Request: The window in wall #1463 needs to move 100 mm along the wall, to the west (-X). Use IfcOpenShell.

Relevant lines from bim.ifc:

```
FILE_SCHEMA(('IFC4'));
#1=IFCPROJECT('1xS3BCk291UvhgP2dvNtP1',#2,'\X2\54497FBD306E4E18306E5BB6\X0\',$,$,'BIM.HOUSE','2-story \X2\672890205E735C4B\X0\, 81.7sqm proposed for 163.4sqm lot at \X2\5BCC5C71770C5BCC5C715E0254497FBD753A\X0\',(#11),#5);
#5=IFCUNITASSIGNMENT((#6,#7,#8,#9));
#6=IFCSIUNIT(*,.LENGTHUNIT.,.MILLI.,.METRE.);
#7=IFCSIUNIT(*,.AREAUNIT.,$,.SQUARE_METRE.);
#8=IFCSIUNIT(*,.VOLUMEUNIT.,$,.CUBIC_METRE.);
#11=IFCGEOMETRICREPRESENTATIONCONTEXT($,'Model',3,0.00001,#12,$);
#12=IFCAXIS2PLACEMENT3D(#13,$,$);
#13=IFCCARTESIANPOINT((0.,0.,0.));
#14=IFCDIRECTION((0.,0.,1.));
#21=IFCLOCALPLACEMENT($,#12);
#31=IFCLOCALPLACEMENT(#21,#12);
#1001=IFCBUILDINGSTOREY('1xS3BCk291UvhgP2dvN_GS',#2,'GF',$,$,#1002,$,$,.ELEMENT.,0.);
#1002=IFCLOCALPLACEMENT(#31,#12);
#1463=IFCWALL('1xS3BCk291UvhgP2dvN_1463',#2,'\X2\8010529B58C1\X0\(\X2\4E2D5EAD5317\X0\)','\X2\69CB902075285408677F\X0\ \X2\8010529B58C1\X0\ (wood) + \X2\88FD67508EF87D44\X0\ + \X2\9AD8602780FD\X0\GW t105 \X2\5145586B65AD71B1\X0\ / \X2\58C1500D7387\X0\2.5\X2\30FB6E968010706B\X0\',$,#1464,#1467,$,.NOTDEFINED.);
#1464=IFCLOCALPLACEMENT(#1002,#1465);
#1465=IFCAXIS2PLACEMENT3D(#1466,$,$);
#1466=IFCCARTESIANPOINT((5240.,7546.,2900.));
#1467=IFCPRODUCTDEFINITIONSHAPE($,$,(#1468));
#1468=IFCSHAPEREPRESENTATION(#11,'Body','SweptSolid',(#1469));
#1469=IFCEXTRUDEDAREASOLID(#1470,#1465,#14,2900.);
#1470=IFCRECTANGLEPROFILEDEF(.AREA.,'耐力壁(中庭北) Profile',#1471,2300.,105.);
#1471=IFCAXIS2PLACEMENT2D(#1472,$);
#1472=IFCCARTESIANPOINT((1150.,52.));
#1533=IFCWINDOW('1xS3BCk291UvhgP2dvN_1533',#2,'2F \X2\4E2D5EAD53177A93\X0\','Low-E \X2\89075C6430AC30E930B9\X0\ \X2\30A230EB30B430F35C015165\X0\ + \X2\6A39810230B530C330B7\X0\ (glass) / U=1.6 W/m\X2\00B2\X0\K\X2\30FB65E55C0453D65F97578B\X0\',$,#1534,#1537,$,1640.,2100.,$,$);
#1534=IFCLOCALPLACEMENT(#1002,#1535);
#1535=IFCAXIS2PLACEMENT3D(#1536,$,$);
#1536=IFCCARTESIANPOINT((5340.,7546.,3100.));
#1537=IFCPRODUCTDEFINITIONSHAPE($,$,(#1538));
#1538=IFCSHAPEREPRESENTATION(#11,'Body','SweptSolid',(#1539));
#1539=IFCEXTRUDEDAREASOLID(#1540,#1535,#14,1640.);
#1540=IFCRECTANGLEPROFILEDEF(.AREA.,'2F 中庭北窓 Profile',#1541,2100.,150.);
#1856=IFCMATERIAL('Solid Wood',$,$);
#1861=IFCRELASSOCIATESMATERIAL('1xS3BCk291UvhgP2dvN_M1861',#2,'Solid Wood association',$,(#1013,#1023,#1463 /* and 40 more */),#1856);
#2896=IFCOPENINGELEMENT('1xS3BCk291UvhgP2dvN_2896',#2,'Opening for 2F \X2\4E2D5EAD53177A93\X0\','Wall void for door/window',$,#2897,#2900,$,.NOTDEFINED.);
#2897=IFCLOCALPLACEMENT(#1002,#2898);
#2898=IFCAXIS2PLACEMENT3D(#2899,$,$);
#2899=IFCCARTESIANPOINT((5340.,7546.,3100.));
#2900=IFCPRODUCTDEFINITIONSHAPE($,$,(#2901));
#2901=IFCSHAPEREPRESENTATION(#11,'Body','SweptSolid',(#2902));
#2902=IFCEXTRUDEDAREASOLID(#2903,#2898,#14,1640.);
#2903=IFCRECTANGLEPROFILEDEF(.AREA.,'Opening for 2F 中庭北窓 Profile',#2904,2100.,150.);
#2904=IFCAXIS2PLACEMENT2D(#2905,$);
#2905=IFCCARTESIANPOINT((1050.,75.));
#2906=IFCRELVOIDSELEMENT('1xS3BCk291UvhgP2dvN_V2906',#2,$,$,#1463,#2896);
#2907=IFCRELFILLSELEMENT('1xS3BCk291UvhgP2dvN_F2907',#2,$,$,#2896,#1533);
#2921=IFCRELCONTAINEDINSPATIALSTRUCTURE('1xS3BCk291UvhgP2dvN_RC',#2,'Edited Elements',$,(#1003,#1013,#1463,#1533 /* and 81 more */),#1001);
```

```python
import ifcopenshell
import ifcopenshell.api.geometry
import ifcopenshell.util.placement
import ifcopenshell.util.unit

model = ifcopenshell.open("bim.ifc")
unit_scale = ifcopenshell.util.unit.calculate_unit_scale(model)

window = model.by_id(1533)
opening = window.FillsVoids[0].RelatingOpeningElement
wall = opening.VoidsElements[0].RelatingBuildingElement

wall_matrix = ifcopenshell.util.placement.get_local_placement(wall.ObjectPlacement)
shift = wall_matrix[:3, 0] * -0.1 / unit_scale
before = ifcopenshell.util.placement.get_local_placement(window.ObjectPlacement)[:3, 3].copy()

# The window is not placed relative to its opening, so move both.
for product in (opening, window):
    matrix = ifcopenshell.util.placement.get_local_placement(product.ObjectPlacement)
    matrix[:3, 3] += shift
    ifcopenshell.api.geometry.edit_object_placement(model, product=product, matrix=matrix, is_si=False)

after = ifcopenshell.util.placement.get_local_placement(window.ObjectPlacement)[:3, 3]
print("window moved by", (after - before).round(3) + 0.0)

model.write("bim_updated.ifc")
```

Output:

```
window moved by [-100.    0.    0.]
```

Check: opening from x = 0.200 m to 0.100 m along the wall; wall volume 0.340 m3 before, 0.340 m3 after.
